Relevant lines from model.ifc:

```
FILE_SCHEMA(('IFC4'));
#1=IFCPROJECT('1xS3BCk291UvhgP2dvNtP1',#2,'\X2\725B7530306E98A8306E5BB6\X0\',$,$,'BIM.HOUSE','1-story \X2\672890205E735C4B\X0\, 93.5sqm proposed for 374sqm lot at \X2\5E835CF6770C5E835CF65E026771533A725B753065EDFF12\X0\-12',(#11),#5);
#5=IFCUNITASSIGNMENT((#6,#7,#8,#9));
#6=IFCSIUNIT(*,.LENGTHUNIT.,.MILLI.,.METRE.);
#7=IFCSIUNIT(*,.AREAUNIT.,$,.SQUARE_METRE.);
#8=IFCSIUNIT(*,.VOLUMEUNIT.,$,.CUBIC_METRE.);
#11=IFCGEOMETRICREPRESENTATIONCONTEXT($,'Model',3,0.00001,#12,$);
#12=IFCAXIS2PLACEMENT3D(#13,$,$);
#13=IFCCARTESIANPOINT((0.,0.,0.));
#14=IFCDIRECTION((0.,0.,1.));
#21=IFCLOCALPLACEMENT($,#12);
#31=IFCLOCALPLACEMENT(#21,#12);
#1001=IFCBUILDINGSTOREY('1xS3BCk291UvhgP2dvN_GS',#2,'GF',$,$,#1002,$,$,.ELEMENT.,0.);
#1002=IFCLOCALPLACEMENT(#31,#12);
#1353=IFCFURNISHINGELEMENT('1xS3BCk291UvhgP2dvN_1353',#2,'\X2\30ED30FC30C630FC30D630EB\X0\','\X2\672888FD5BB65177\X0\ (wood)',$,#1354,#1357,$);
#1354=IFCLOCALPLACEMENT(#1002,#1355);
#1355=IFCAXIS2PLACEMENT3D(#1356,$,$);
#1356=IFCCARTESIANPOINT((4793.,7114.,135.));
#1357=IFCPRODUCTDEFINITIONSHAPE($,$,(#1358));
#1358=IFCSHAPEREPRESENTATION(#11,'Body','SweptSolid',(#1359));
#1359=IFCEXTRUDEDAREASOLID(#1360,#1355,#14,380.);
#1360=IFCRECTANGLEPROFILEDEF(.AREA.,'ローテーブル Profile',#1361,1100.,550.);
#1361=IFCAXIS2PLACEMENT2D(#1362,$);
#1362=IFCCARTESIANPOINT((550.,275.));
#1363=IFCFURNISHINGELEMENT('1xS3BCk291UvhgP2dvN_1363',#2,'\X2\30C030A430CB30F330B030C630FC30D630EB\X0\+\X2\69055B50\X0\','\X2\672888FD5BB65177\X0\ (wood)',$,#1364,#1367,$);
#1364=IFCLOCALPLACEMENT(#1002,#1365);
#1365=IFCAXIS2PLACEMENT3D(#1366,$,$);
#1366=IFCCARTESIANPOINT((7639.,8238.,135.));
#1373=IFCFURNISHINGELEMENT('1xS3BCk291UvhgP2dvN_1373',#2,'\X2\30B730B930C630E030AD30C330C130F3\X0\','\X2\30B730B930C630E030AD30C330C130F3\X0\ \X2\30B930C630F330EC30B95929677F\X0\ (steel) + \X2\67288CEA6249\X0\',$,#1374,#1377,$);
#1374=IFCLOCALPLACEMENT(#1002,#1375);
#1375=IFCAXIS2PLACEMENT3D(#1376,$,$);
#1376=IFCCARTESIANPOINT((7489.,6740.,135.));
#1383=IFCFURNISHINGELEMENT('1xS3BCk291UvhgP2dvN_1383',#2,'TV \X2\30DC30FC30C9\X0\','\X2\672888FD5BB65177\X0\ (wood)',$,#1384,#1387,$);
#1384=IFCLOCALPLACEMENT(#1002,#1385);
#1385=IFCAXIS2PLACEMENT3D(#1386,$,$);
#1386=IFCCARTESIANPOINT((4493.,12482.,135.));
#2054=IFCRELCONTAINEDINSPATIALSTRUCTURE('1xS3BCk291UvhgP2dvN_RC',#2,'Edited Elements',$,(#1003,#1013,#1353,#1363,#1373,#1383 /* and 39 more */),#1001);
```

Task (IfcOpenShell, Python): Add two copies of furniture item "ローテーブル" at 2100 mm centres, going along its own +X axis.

```python
import ifcopenshell
import ifcopenshell.api.geometry
import ifcopenshell.api.root
import ifcopenshell.util.element
import ifcopenshell.util.placement

model = ifcopenshell.open("model.ifc")


def reuse_history(source, copy):
    """copy_class also copies each property set's owner history, people and application; keep the originals."""
    for rel in copy.IsDefinedBy:
        if rel.is_a("IfcRelDefinesByProperties") and (history := rel.RelatingPropertyDefinition.OwnerHistory):
            rel.RelatingPropertyDefinition.OwnerHistory = source.OwnerHistory
            ifcopenshell.util.element.remove_deep2(model, history)


source = model.by_id(1353)
base = ifcopenshell.util.placement.get_local_placement(source.ObjectPlacement)
step = base[:3, 0] * 2100.0

for i in range(1, 3):
    copy = ifcopenshell.api.root.copy_class(model, product=source)
    copy.Representation = ifcopenshell.util.element.copy_deep(
        model, source.Representation, exclude=["IfcGeometricRepresentationContext", "IfcRepresentationMap"]
    )
    reuse_history(source, copy)
    matrix = base.copy()
    matrix[:3, 3] += i * step
    print("added at", matrix[:3, 3].round(3) + 0.0)
    ifcopenshell.api.geometry.edit_object_placement(model, product=copy, matrix=matrix, is_si=False)

model.write("model_edited.ifc")
```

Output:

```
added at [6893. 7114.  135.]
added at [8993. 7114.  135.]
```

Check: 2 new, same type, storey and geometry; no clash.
